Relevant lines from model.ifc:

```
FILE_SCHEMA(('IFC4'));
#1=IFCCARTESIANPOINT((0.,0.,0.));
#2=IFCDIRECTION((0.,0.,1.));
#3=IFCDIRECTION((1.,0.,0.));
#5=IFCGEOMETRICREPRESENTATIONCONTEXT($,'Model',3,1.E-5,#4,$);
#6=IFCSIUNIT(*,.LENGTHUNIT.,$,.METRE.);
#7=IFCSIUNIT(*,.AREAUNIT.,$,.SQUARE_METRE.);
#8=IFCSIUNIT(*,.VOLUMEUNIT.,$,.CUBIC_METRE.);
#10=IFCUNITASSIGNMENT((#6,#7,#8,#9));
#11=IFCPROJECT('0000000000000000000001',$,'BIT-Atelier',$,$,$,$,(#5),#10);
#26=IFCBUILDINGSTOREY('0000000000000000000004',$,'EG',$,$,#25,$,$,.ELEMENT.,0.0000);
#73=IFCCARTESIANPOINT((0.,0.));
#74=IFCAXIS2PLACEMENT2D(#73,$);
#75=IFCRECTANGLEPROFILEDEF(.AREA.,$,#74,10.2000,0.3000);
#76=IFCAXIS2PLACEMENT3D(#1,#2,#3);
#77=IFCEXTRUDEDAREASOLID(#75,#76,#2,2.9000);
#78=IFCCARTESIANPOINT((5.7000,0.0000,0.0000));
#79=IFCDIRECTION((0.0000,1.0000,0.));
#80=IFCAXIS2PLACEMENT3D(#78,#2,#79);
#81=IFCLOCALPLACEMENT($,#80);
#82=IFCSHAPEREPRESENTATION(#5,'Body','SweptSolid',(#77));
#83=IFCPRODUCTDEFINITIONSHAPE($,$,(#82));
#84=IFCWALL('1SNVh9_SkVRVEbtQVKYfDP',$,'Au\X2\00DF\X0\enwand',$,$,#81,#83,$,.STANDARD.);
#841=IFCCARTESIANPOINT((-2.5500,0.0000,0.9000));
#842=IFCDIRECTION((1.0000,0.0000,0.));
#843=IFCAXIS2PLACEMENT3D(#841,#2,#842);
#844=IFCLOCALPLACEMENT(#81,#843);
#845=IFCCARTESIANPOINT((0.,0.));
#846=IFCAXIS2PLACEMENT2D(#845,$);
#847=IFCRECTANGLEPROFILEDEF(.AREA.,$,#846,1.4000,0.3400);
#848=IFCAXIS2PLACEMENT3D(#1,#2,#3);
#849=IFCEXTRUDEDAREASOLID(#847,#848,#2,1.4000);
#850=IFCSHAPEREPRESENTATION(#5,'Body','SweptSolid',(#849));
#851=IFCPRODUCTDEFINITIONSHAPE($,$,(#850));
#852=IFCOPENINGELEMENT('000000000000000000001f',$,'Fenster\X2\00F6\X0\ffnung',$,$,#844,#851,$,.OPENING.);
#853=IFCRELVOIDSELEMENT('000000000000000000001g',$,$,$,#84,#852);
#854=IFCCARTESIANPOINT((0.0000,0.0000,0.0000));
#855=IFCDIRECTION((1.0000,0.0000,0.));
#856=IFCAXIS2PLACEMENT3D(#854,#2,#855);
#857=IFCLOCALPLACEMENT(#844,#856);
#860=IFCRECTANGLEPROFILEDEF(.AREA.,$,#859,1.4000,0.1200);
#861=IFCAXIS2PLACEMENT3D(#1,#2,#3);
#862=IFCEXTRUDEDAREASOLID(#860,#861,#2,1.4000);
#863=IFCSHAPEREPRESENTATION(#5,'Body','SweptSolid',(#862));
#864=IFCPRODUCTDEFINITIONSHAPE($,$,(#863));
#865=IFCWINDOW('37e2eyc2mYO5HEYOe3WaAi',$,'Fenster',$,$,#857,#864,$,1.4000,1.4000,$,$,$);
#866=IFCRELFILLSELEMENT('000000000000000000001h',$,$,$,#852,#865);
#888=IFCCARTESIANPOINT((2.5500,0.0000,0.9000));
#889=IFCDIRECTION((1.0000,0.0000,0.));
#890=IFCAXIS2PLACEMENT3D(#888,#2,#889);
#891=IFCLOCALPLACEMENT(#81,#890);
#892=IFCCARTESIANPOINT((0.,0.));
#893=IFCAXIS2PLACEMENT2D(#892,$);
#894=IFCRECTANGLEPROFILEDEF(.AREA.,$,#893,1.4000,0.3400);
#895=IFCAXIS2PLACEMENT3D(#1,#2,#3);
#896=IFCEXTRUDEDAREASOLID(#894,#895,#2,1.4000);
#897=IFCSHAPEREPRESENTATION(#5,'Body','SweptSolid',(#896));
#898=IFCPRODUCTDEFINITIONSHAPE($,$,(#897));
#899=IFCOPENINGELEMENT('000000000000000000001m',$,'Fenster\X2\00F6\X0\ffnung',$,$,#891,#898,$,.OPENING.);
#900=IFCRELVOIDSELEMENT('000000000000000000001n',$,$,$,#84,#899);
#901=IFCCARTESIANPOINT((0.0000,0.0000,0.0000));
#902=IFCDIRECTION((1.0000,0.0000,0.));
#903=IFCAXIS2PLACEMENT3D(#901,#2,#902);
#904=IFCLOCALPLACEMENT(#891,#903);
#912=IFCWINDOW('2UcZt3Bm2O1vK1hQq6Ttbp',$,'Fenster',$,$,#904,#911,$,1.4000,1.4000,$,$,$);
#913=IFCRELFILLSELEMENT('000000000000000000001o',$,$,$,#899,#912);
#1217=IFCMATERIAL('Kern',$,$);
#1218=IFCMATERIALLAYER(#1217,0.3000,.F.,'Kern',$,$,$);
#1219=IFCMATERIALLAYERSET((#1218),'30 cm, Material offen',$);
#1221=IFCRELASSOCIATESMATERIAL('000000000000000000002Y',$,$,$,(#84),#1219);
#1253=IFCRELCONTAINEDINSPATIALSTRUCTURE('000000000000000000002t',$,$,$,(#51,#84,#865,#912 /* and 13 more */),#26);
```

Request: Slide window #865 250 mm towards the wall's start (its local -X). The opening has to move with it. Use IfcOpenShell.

```python
import ifcopenshell
import ifcopenshell.api.geometry
import ifcopenshell.util.placement

model = ifcopenshell.open("model.ifc")

window = model.by_guid("37e2eyc2mYO5HEYOe3WaAi")
opening = window.FillsVoids[0].RelatingOpeningElement
wall = opening.VoidsElements[0].RelatingBuildingElement

wall_matrix = ifcopenshell.util.placement.get_local_placement(wall.ObjectPlacement)
shift = wall_matrix[:3, 0] * -0.25
before = ifcopenshell.util.placement.get_local_placement(window.ObjectPlacement)[:3, 3].copy()

# The window is placed relative to its opening, so it follows when the opening moves.
matrix = ifcopenshell.util.placement.get_local_placement(opening.ObjectPlacement)
matrix[:3, 3] += shift
ifcopenshell.api.geometry.edit_object_placement(
    model, product=opening, matrix=matrix, is_si=False, should_transform_children=True
)

after = ifcopenshell.util.placement.get_local_placement(window.ObjectPlacement)[:3, 3]
print("window moved by", (after - before).round(3) + 0.0)

model.write("model_updated.ifc")
```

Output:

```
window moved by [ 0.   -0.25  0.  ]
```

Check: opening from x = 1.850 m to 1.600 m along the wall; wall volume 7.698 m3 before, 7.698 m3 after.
